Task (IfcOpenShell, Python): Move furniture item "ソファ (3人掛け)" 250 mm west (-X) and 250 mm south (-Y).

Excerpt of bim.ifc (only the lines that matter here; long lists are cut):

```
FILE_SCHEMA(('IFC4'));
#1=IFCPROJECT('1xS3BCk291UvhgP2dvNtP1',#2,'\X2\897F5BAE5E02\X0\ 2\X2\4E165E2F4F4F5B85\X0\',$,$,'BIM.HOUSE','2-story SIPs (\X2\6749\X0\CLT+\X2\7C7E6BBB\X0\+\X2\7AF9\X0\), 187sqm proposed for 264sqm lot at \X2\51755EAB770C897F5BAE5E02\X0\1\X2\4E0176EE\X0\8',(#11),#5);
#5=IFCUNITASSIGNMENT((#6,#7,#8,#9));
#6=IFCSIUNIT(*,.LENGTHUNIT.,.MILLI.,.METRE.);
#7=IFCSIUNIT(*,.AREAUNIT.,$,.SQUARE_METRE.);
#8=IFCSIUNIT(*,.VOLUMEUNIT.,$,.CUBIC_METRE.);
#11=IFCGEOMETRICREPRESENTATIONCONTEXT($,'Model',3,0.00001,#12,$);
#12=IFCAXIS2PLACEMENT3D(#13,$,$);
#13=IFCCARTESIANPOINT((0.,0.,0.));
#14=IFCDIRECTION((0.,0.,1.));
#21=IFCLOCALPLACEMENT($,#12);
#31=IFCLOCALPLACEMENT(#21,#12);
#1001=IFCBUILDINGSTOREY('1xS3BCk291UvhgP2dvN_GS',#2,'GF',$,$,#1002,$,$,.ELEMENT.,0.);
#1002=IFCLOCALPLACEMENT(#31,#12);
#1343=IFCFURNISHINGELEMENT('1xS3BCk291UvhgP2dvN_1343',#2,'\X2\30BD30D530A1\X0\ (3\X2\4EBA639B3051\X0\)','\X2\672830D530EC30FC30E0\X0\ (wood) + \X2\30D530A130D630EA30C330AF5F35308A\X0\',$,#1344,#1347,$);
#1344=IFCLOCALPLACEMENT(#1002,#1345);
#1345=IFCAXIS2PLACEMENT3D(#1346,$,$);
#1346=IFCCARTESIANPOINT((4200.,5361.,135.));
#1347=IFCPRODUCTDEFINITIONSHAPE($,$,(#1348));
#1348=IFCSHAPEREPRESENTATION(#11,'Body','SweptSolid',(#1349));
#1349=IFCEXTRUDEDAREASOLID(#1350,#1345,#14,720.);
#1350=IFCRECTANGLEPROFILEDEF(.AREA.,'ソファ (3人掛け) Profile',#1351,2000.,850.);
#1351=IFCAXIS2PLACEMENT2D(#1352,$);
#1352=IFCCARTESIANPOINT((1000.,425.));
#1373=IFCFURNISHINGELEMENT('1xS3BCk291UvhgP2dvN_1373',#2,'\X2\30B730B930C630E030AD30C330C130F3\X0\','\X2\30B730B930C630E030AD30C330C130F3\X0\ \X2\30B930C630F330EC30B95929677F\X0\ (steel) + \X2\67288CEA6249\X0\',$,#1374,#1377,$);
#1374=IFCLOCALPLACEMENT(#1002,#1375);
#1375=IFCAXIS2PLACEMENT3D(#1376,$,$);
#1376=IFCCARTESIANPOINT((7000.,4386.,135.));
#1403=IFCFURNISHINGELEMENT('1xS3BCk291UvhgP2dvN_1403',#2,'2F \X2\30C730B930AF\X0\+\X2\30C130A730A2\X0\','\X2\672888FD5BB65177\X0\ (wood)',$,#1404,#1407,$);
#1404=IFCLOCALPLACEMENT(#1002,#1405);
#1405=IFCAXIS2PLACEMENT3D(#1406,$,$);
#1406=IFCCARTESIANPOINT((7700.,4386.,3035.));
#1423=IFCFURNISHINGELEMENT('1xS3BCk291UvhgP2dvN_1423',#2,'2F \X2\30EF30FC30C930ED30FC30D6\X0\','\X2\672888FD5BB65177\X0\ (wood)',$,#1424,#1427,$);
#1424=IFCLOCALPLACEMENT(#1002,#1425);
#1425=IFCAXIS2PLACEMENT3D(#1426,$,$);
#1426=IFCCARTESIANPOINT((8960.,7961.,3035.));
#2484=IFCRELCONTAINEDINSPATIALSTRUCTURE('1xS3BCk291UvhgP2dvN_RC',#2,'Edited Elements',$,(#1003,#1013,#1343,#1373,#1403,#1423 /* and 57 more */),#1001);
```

```python
import ifcopenshell
import ifcopenshell.api.geometry
import ifcopenshell.util.placement
import ifcopenshell.util.unit

model = ifcopenshell.open("bim.ifc")
unit_scale = ifcopenshell.util.unit.calculate_unit_scale(model)

item = model.by_id(1343)
matrix = ifcopenshell.util.placement.get_local_placement(item.ObjectPlacement)
matrix[0, 3] -= 0.25 / unit_scale
matrix[1, 3] -= 0.25 / unit_scale
ifcopenshell.api.geometry.edit_object_placement(model, product=item, matrix=matrix, is_si=False)

print(ifcopenshell.util.placement.get_local_placement(item.ObjectPlacement).round(3) + 0.0)

model.write("bim_rev.ifc")
```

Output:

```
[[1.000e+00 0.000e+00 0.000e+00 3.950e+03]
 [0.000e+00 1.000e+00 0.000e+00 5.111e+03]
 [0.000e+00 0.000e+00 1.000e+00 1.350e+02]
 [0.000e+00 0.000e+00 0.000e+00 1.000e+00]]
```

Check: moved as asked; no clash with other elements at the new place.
